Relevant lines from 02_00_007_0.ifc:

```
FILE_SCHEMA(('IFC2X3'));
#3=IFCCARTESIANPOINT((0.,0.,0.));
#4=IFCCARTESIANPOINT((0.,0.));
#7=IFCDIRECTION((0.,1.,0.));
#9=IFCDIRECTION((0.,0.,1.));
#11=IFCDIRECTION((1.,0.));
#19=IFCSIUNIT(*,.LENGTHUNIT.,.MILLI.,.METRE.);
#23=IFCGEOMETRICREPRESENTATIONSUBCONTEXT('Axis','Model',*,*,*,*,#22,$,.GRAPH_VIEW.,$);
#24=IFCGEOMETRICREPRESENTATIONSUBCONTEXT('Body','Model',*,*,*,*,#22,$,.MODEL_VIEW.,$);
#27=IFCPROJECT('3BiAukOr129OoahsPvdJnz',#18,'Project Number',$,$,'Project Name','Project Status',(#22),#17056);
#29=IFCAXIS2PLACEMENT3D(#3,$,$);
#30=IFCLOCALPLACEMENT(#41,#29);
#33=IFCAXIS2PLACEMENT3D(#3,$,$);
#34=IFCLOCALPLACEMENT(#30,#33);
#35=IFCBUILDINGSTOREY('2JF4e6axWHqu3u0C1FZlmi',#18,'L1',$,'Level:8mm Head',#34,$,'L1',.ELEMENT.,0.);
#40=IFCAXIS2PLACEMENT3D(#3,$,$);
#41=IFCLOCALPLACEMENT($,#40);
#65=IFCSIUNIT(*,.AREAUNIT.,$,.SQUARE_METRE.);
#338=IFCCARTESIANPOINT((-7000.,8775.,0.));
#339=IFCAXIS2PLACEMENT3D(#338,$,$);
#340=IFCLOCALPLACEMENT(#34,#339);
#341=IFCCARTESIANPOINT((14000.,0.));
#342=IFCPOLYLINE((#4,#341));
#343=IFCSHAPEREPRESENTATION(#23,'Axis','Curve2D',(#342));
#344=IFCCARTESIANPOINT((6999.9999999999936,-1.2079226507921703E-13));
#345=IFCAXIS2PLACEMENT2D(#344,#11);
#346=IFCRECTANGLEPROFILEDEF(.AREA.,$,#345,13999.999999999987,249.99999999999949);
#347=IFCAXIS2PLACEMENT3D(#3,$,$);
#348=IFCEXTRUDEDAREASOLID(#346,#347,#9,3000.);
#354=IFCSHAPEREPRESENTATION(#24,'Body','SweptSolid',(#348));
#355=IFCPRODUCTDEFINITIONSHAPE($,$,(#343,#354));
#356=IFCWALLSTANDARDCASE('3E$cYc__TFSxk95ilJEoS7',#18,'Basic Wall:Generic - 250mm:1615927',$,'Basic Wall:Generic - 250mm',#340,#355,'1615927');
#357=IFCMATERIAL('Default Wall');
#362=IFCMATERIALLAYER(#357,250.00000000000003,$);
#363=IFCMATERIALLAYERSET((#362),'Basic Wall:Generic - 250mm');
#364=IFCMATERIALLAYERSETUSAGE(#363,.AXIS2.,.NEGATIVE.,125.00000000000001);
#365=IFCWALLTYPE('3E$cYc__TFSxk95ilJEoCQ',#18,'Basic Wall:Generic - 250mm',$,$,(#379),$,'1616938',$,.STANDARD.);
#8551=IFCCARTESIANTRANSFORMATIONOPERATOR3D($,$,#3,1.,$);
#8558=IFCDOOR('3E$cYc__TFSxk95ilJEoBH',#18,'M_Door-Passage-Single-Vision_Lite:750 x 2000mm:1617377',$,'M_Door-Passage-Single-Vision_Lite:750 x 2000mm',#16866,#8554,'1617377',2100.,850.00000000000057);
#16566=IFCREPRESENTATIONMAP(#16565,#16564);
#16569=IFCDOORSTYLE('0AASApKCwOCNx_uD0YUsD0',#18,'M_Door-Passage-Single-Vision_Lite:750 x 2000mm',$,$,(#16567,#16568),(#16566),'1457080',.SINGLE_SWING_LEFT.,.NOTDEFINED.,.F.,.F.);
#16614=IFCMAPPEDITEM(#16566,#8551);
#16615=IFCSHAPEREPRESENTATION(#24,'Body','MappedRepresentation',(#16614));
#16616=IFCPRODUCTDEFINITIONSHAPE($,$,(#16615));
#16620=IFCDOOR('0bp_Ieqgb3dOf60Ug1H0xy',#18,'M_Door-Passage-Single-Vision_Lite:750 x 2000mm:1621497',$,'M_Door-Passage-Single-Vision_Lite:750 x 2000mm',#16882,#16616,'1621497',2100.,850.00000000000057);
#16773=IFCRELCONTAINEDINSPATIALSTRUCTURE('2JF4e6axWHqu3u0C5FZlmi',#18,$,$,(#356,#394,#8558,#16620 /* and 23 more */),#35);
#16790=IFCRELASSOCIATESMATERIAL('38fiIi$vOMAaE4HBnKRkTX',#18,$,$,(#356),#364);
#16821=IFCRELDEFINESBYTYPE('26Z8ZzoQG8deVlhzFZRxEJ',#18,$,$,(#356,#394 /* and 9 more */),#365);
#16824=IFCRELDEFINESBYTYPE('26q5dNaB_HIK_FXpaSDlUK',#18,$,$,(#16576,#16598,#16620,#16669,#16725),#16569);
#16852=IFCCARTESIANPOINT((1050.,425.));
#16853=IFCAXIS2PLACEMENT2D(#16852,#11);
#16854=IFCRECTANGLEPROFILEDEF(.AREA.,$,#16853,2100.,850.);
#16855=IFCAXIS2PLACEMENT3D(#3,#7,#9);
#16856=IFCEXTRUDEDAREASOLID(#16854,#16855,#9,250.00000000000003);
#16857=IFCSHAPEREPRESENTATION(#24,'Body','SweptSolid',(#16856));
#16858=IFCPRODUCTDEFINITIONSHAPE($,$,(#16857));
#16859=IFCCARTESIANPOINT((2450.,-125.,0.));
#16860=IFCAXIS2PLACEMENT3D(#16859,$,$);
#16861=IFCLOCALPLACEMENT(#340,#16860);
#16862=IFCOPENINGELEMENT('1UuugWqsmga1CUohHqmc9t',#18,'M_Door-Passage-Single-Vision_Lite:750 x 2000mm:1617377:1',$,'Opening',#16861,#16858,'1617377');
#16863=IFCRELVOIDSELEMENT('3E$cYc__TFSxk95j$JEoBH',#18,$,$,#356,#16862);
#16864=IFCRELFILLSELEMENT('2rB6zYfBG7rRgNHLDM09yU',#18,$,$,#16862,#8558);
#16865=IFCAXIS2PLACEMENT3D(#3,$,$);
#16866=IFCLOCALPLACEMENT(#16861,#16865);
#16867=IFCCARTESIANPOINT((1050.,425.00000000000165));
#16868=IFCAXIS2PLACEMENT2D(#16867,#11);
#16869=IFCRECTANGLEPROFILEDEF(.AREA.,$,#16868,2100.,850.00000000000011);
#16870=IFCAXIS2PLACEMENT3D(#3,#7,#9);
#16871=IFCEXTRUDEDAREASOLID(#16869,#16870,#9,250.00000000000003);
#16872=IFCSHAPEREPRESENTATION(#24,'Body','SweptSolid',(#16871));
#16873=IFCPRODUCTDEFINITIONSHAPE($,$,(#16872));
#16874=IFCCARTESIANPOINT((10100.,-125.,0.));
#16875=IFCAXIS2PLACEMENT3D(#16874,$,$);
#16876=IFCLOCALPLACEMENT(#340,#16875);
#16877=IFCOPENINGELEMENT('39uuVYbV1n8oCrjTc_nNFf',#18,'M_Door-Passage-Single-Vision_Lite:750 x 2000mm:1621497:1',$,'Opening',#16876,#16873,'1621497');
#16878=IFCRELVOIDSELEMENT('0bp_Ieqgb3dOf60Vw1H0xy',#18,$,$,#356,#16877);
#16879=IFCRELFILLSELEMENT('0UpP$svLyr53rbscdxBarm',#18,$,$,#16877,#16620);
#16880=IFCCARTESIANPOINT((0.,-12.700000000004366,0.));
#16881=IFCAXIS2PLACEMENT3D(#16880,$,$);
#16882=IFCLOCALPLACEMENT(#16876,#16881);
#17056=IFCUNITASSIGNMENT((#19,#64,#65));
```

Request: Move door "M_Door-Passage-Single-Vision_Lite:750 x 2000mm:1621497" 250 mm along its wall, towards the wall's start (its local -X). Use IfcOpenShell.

```python
import ifcopenshell
import ifcopenshell.api.geometry
import ifcopenshell.util.placement
import ifcopenshell.util.unit

model = ifcopenshell.open("02_00_007_0.ifc")
unit_scale = ifcopenshell.util.unit.calculate_unit_scale(model)

door = model.by_guid("0bp_Ieqgb3dOf60Ug1H0xy")
opening = door.FillsVoids[0].RelatingOpeningElement
wall = opening.VoidsElements[0].RelatingBuildingElement

wall_matrix = ifcopenshell.util.placement.get_local_placement(wall.ObjectPlacement)
shift = wall_matrix[:3, 0] * -0.25 / unit_scale
before = ifcopenshell.util.placement.get_local_placement(door.ObjectPlacement)[:3, 3].copy()

# The door is placed relative to its opening, so it follows when the opening moves.
matrix = ifcopenshell.util.placement.get_local_placement(opening.ObjectPlacement)
matrix[:3, 3] += shift
ifcopenshell.api.geometry.edit_object_placement(
    model, product=opening, matrix=matrix, is_si=False, should_transform_children=True
)

after = ifcopenshell.util.placement.get_local_placement(door.ObjectPlacement)[:3, 3]
print("door moved by", (after - before).round(3) + 0.0)

model.write("02_00_007_0-out.ifc")
```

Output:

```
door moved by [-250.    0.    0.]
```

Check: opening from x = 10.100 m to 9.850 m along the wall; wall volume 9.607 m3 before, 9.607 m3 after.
